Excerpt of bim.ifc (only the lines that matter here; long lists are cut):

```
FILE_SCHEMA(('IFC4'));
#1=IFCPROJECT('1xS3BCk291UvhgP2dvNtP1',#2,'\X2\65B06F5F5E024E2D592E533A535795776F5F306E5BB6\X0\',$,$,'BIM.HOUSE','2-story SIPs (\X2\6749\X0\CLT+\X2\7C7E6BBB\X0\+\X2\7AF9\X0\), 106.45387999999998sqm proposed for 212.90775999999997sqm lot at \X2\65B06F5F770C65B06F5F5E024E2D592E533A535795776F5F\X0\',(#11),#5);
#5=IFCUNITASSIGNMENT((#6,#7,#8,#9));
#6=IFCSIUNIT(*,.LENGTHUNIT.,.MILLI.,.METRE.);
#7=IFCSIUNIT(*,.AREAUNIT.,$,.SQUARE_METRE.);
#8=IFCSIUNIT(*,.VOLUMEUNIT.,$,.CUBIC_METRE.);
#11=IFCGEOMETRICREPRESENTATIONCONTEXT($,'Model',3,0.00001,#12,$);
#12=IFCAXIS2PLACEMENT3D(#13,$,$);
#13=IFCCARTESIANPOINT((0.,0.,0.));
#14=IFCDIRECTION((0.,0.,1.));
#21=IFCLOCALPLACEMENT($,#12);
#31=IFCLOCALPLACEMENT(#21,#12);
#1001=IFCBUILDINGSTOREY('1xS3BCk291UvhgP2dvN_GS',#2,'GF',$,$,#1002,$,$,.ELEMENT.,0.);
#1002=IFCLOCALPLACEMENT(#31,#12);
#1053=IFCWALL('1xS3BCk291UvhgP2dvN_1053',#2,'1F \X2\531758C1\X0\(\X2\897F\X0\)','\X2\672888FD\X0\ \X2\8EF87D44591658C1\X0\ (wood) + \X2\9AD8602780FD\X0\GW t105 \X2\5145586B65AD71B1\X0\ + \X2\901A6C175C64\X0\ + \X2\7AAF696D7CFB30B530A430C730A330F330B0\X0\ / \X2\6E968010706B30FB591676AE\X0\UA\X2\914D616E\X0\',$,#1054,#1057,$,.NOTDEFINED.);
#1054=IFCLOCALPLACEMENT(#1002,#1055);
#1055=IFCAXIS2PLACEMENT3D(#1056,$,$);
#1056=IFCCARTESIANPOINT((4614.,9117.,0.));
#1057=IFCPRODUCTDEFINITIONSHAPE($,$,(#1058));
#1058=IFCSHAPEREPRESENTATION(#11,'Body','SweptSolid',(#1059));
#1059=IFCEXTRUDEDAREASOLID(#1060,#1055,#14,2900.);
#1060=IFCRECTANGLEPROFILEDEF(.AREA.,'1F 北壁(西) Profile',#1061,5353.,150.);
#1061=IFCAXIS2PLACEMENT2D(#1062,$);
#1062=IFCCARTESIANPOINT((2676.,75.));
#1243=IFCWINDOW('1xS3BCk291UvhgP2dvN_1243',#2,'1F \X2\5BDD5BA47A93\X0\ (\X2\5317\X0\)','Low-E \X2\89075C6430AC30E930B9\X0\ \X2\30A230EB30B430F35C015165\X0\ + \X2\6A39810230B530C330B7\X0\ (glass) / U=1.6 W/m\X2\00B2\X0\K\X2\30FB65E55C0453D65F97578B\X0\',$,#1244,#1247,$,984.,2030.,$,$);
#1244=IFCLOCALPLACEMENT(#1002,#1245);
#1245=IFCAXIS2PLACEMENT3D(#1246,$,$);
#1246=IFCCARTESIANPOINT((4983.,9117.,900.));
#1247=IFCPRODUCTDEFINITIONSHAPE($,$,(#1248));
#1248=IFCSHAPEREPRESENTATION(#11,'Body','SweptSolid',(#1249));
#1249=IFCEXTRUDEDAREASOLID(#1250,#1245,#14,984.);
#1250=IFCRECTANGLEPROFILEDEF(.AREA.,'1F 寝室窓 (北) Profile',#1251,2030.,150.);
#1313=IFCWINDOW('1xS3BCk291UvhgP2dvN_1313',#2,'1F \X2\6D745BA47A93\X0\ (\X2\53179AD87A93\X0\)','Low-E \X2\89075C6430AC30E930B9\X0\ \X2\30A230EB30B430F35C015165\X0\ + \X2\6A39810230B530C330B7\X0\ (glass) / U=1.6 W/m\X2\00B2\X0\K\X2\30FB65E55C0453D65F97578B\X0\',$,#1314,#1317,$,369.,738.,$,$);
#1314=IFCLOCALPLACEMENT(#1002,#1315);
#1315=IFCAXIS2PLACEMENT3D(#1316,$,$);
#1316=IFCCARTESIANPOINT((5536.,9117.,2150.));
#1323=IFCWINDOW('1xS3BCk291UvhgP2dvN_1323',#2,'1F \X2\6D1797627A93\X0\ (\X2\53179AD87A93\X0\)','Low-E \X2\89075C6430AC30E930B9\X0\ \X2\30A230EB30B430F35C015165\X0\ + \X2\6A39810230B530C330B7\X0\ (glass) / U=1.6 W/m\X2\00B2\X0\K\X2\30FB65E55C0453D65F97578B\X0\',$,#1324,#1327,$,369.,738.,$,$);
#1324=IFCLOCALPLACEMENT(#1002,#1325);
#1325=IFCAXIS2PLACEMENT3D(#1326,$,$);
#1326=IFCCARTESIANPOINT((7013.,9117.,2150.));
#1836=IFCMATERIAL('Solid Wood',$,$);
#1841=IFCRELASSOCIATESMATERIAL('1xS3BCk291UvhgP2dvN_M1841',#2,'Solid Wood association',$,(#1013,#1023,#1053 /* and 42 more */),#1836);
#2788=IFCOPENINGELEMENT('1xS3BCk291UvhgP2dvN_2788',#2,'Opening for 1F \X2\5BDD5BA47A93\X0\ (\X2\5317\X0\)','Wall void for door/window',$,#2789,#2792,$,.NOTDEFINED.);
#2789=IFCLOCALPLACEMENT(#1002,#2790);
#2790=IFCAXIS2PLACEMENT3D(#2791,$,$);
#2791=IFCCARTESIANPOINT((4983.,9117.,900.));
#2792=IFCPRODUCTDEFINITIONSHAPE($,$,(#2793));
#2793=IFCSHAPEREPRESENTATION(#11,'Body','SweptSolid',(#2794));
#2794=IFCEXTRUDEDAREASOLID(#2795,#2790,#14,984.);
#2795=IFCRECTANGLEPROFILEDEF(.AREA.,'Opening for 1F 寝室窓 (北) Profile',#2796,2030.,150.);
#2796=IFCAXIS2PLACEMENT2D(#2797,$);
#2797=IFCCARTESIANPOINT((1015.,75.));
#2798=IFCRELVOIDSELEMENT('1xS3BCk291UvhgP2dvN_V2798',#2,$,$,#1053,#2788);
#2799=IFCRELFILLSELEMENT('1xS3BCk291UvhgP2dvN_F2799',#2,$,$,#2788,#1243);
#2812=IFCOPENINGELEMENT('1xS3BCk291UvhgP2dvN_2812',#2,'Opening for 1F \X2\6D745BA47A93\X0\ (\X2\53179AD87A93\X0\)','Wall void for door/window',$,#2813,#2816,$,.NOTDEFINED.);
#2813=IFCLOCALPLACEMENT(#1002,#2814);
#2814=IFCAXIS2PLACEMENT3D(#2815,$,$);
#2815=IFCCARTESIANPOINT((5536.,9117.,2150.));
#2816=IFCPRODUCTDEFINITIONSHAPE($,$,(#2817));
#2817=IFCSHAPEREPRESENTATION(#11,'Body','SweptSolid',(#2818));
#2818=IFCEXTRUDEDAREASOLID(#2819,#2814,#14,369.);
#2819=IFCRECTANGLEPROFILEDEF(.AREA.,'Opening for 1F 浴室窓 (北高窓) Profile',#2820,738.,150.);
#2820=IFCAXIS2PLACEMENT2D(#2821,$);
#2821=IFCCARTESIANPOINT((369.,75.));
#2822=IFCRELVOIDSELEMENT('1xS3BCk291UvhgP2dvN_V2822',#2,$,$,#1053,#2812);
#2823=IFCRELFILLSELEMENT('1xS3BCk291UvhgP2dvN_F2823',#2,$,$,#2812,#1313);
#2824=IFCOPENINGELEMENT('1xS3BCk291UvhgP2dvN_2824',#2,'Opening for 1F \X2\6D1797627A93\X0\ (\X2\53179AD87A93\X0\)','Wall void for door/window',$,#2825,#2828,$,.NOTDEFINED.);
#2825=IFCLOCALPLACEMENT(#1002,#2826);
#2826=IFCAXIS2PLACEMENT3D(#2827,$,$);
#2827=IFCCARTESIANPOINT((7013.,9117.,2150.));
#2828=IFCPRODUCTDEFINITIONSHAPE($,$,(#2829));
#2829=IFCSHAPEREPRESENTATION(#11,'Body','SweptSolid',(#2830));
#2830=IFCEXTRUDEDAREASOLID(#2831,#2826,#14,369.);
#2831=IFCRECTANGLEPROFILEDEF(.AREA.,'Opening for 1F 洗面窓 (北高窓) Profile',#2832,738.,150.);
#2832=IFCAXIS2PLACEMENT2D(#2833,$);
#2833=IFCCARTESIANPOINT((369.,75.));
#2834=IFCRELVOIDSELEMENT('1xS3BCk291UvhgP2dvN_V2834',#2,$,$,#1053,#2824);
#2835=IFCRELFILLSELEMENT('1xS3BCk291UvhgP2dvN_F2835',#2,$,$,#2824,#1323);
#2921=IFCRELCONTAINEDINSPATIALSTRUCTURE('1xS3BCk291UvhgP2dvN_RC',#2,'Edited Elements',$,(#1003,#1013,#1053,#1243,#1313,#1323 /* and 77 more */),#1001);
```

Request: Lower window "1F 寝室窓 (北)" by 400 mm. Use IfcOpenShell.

```python
import numpy as np
import ifcopenshell
import ifcopenshell.api.geometry
import ifcopenshell.util.placement
import ifcopenshell.util.unit

model = ifcopenshell.open("bim.ifc")
unit_scale = ifcopenshell.util.unit.calculate_unit_scale(model)

window = model.by_id(1243)
opening = window.FillsVoids[0].RelatingOpeningElement
dz = -0.4 / unit_scale

shift = np.array([0.0, 0.0, dz])
# The window is not placed relative to its opening, so move both.
for product in (opening, window):
    matrix = ifcopenshell.util.placement.get_local_placement(product.ObjectPlacement)
    matrix[:3, 3] += shift
    ifcopenshell.api.geometry.edit_object_placement(model, product=product, matrix=matrix, is_si=False)

print(f"moved by {dz * unit_scale:+.3f} m")

model.write("bim_edited.ifc")
```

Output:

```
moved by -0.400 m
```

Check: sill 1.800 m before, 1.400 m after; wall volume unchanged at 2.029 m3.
